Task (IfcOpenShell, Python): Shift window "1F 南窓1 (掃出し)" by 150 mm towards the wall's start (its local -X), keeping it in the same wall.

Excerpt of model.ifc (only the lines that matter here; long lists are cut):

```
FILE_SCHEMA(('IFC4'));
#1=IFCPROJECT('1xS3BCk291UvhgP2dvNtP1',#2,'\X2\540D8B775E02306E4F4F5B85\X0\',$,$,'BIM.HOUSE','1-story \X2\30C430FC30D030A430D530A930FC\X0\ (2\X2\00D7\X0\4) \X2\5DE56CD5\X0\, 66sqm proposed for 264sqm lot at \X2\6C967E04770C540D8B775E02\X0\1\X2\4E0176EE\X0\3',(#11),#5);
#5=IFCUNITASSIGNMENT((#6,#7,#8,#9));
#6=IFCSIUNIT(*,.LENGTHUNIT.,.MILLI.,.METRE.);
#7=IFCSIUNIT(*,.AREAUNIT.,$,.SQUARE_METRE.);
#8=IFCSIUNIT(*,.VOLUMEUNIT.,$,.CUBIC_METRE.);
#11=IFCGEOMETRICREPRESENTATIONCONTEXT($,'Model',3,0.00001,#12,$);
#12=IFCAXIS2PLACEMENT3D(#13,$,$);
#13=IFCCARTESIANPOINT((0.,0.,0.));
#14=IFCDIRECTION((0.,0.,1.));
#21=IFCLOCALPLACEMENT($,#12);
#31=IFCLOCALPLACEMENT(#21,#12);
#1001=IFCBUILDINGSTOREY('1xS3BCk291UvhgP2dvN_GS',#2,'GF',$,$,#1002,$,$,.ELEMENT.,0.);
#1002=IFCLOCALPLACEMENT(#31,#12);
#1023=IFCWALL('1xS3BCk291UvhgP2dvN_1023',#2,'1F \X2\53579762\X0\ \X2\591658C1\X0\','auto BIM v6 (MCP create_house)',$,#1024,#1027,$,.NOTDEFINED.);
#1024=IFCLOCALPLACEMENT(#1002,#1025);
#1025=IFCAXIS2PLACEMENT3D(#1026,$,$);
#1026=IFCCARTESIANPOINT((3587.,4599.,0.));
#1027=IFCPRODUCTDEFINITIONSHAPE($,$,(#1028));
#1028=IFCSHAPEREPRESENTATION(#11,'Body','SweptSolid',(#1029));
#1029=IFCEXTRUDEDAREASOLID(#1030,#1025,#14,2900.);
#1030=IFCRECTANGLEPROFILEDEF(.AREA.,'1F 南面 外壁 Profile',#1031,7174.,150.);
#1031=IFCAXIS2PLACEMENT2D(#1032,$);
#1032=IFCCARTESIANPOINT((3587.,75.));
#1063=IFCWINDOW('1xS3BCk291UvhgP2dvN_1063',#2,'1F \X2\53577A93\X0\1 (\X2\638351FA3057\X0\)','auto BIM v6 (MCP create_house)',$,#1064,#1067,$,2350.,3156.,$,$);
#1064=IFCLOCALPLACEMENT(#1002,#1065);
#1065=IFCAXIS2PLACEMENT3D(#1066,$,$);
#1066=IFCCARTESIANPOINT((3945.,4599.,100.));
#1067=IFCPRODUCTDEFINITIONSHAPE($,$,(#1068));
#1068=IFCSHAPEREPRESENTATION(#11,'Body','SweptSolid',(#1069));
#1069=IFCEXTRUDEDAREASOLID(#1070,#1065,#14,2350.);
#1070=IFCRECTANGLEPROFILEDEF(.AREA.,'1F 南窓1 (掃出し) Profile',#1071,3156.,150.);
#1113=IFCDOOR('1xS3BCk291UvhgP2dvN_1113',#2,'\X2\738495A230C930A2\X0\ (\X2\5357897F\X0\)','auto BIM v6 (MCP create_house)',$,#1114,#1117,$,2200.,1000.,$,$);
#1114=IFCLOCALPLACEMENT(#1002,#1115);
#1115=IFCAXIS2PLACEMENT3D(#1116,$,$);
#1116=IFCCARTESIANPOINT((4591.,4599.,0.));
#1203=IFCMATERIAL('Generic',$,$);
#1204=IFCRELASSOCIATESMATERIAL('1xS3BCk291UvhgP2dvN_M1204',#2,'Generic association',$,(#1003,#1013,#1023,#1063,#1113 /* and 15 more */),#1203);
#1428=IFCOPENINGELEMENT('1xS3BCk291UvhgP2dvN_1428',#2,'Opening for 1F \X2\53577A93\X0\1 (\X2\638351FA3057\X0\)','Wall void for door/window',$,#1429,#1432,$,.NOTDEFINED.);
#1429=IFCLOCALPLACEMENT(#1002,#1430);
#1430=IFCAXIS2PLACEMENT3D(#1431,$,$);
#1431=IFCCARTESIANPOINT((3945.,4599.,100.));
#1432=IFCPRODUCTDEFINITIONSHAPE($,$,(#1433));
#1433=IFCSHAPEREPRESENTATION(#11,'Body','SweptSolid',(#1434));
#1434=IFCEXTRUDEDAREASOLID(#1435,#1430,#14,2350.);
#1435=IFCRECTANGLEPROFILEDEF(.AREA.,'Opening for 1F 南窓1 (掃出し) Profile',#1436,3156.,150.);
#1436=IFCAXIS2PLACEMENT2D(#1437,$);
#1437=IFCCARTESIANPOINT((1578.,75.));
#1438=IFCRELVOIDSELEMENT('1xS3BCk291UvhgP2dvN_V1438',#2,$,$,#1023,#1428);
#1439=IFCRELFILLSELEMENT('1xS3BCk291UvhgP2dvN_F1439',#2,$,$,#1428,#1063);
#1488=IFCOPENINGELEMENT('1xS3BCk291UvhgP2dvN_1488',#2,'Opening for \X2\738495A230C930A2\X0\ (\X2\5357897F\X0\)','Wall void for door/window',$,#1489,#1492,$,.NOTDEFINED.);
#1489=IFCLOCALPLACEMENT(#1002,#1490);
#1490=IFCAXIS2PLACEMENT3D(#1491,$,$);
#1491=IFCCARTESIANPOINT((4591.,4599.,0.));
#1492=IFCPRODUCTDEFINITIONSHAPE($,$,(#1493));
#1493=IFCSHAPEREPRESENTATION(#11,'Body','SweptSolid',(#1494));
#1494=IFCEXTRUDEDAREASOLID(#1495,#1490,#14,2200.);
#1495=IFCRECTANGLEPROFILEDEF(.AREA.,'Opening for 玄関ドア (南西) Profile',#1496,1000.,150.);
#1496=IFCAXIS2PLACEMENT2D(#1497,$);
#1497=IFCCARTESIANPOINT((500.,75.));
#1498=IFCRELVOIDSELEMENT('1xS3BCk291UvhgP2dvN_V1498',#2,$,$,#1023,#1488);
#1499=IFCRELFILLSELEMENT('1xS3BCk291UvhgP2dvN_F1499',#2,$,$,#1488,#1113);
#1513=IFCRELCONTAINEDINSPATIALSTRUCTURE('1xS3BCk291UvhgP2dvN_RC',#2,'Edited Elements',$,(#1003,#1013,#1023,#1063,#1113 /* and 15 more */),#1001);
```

```python
import ifcopenshell
import ifcopenshell.api.geometry
import ifcopenshell.util.placement
import ifcopenshell.util.unit

model = ifcopenshell.open("model.ifc")
unit_scale = ifcopenshell.util.unit.calculate_unit_scale(model)

window = model.by_guid("1xS3BCk291UvhgP2dvN_1063")
opening = window.FillsVoids[0].RelatingOpeningElement
wall = opening.VoidsElements[0].RelatingBuildingElement

wall_matrix = ifcopenshell.util.placement.get_local_placement(wall.ObjectPlacement)
shift = wall_matrix[:3, 0] * -0.15 / unit_scale
before = ifcopenshell.util.placement.get_local_placement(window.ObjectPlacement)[:3, 3].copy()

# The window is not placed relative to its opening, so move both.
for product in (opening, window):
    matrix = ifcopenshell.util.placement.get_local_placement(product.ObjectPlacement)
    matrix[:3, 3] += shift
    ifcopenshell.api.geometry.edit_object_placement(model, product=product, matrix=matrix, is_si=False)

after = ifcopenshell.util.placement.get_local_placement(window.ObjectPlacement)[:3, 3]
print("window moved by", (after - before).round(3) + 0.0)

model.write("model_v2.ifc")
```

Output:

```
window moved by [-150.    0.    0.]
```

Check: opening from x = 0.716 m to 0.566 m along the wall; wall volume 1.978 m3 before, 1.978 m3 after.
